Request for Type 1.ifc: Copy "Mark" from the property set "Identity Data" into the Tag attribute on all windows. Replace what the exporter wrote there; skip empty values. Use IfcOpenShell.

First a look at what the model holds.

```python
import ifcopenshell
import ifcopenshell.util.element

model = ifcopenshell.open("Type 1.ifc")
print(model.schema)
windows = model.by_type("IfcWindow")
print(len(windows), "windows")
for e in windows[:8]:
    source = ifcopenshell.util.element.get_pset(e, "Identity Data", "Mark")
    target = e.Tag
    print(e.id(), repr(source), repr(target), sep=" | ")
```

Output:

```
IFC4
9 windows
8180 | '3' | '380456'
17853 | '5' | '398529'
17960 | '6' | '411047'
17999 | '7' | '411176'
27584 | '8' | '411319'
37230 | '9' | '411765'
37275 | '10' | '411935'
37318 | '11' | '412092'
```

```python
import ifcopenshell
import ifcopenshell.util.element

model = ifcopenshell.open("Type 1.ifc")

count = 0
for e in model.by_type("IfcWindow"):
    value = ifcopenshell.util.element.get_pset(e, "Identity Data", "Mark")
    current = e.Tag
    if not value or not value.strip() or current == value:
        continue
    e.Tag = value
    count += 1

print(count, "windows updated")

model.write("Type 1_rev.ifc")
```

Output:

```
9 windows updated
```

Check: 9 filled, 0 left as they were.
